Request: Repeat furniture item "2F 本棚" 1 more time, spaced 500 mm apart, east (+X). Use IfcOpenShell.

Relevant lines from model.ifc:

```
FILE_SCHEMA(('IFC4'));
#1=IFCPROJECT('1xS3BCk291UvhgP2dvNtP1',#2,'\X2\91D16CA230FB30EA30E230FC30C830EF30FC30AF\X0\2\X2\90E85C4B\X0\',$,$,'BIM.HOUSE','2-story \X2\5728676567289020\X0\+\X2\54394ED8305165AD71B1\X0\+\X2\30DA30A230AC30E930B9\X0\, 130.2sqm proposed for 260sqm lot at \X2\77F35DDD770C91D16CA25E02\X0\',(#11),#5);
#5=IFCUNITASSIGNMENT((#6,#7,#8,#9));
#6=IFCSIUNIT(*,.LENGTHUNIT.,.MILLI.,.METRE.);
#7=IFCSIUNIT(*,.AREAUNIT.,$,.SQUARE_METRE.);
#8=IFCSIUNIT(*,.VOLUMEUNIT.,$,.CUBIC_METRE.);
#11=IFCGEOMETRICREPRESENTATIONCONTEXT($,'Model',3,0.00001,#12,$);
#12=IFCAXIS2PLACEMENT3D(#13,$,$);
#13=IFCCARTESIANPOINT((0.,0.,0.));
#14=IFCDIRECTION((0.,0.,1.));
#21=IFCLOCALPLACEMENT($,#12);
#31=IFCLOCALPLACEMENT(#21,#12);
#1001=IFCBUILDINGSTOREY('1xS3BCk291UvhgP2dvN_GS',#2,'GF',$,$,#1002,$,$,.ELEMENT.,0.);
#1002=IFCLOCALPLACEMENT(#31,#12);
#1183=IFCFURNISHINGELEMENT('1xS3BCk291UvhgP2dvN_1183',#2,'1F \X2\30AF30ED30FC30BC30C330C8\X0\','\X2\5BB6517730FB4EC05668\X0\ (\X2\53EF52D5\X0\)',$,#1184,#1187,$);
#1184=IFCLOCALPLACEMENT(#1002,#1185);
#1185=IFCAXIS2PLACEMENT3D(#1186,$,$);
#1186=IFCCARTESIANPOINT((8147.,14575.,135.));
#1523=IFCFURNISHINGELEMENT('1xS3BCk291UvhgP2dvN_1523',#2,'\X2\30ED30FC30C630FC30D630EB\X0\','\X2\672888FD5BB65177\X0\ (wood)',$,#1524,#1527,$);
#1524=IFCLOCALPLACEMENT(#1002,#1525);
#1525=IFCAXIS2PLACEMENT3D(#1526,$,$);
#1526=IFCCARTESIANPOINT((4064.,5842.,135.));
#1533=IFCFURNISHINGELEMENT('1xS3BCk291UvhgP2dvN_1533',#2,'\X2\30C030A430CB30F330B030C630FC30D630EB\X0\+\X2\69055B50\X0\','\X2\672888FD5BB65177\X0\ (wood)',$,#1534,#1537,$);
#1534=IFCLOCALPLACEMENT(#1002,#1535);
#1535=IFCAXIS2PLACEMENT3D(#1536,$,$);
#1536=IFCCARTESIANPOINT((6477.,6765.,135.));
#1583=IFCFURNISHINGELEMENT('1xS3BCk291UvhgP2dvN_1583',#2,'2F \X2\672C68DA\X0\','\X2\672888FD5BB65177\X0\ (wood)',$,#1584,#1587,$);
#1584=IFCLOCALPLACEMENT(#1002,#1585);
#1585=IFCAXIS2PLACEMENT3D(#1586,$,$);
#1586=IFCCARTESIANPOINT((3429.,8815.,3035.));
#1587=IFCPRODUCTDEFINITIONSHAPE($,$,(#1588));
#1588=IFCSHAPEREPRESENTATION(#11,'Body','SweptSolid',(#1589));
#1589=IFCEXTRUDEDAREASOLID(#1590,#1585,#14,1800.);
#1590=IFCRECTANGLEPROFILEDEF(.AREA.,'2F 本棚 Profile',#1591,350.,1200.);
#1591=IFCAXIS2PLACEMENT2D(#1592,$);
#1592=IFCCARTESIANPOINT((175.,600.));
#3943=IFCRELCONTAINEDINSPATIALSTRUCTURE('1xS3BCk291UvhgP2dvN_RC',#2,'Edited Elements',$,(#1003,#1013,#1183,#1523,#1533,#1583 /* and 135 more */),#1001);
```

```python
import numpy as np
import ifcopenshell
import ifcopenshell.api.geometry
import ifcopenshell.api.root
import ifcopenshell.util.element
import ifcopenshell.util.placement

model = ifcopenshell.open("model.ifc")


def reuse_history(source, copy):
    """copy_class also copies each property set's owner history, people and application; keep the originals."""
    for rel in copy.IsDefinedBy:
        if rel.is_a("IfcRelDefinesByProperties") and (history := rel.RelatingPropertyDefinition.OwnerHistory):
            rel.RelatingPropertyDefinition.OwnerHistory = source.OwnerHistory
            ifcopenshell.util.element.remove_deep2(model, history)


source = model.by_guid("1xS3BCk291UvhgP2dvN_1583")
base = ifcopenshell.util.placement.get_local_placement(source.ObjectPlacement)
step = np.array([1.0, 0.0, 0.0]) * 500.0

for i in range(1, 2):
    copy = ifcopenshell.api.root.copy_class(model, product=source)
    copy.Representation = ifcopenshell.util.element.copy_deep(
        model, source.Representation, exclude=["IfcGeometricRepresentationContext", "IfcRepresentationMap"]
    )
    reuse_history(source, copy)
    matrix = base.copy()
    matrix[:3, 3] += i * step
    print("added at", matrix[:3, 3].round(3) + 0.0)
    ifcopenshell.api.geometry.edit_object_placement(model, product=copy, matrix=matrix, is_si=False)

model.write("model_v2.ifc")
```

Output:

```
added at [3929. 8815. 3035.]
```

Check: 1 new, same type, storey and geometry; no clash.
